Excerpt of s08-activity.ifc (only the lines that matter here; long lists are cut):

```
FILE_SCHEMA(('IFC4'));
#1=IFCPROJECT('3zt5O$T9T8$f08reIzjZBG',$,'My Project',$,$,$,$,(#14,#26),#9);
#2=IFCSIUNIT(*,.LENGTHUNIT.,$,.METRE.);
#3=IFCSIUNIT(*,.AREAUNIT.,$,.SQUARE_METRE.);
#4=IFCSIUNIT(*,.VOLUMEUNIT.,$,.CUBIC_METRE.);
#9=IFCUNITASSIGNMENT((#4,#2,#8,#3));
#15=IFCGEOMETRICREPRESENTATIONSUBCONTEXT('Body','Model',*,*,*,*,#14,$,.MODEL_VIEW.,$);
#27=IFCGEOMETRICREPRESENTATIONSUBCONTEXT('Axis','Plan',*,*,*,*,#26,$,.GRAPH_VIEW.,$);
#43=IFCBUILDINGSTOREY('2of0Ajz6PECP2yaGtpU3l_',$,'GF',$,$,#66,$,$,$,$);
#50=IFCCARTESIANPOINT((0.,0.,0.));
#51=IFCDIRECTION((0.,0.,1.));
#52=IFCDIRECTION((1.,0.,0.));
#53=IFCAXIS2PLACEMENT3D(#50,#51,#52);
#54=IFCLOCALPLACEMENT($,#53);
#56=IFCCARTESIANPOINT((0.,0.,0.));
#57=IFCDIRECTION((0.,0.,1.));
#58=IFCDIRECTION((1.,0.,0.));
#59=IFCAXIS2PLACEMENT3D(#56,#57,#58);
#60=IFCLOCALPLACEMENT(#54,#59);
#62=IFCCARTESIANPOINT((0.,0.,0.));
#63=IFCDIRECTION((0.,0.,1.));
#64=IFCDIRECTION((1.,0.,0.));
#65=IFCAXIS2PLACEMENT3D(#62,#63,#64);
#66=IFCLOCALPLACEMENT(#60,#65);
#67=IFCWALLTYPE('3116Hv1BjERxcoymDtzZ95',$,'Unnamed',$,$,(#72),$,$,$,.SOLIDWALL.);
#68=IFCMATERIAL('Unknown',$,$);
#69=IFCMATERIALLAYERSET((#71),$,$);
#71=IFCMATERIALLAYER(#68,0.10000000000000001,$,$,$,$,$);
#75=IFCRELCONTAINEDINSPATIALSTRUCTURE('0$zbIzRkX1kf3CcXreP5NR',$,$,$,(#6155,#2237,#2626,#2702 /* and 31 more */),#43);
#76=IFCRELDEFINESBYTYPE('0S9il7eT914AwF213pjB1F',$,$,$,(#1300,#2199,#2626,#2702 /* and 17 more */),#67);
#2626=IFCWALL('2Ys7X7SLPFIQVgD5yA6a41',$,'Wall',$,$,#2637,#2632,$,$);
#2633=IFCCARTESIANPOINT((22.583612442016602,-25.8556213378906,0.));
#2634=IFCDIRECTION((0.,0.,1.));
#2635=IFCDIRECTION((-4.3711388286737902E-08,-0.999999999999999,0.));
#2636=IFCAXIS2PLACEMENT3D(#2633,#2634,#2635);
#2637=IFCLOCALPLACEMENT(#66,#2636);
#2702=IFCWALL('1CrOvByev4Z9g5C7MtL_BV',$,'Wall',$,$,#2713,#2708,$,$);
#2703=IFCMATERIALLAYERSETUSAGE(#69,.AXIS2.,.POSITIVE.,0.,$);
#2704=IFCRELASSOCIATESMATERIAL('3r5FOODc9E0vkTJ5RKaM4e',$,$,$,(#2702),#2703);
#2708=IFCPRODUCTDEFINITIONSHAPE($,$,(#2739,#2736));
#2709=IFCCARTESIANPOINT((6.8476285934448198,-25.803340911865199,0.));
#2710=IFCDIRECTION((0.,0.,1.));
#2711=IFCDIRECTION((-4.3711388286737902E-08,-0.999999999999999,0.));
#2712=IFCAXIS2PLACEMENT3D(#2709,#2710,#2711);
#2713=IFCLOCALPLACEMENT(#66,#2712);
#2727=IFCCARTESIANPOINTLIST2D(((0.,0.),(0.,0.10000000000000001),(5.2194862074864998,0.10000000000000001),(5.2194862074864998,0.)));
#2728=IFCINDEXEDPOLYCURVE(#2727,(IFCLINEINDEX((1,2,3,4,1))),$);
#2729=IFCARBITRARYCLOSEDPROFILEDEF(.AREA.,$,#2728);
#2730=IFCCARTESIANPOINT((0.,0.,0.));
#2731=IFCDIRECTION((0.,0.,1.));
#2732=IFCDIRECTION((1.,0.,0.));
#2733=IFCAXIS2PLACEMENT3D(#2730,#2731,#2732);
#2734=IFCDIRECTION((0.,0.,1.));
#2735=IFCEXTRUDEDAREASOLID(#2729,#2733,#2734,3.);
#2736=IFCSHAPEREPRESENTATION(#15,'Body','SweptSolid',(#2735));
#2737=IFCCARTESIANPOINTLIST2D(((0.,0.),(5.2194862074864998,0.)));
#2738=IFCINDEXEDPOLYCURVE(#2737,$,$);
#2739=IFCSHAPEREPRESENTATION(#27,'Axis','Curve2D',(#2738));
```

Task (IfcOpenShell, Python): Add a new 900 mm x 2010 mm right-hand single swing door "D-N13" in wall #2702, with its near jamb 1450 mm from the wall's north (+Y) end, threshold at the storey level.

```python
import numpy as np
import ifcopenshell
import ifcopenshell.api.feature
import ifcopenshell.api.geometry
import ifcopenshell.api.root
import ifcopenshell.api.spatial
import ifcopenshell.geom
import ifcopenshell.util.element
import ifcopenshell.util.placement
import ifcopenshell.util.representation
import ifcopenshell.util.shape
import ifcopenshell.util.unit

model = ifcopenshell.open("s08-activity.ifc")
unit_scale = ifcopenshell.util.unit.calculate_unit_scale(model)
settings = ifcopenshell.geom.settings()


def volume(element):
    """Net volume in cubic metres, openings subtracted."""
    shape = ifcopenshell.geom.create_shape(settings, element)
    return ifcopenshell.util.shape.get_volume(shape.geometry)


wall = model.by_guid("1CrOvByev4Z9g5C7MtL_BV")
storey = ifcopenshell.util.element.get_container(wall, ifc_class="IfcBuildingStorey")
context = ifcopenshell.util.representation.get_context(model, "Model", "Body", "MODEL_VIEW")
before = volume(wall)

width, height, from_end, sill = 0.9, 2.01, 1.45, 0.0  # metres

# The wall runs along its own X axis, and the end named is its -X end.
wall_shape = ifcopenshell.geom.create_shape(settings, wall)
x, y, z = ifcopenshell.util.shape.get_vertices(wall_shape.geometry).T
start = x.min() + from_end
face, thickness = float(y.min()), float(y.max() - y.min())
wall_matrix = ifcopenshell.util.placement.get_local_placement(wall.ObjectPlacement)
level = ifcopenshell.util.placement.get_local_placement(storey.ObjectPlacement)[2, 3]


def in_wall(x, y):
    """Placement at x, y metres in the wall's axes, at sill height."""
    matrix = wall_matrix.copy()
    matrix[:, 3] = wall_matrix @ np.array([x / unit_scale, y / unit_scale, 0.0, 1.0])
    matrix[2, 3] = level + sill / unit_scale
    return matrix


# Opening: a box that overshoots both wall faces by 50 mm.
opening = ifcopenshell.api.root.create_entity(model, ifc_class="IfcOpeningElement", predefined_type="OPENING")
box = ifcopenshell.api.geometry.add_wall_representation(
    model, context=context, length=width, height=height, thickness=thickness + 0.1
)
ifcopenshell.api.geometry.assign_representation(model, product=opening, representation=box)
ifcopenshell.api.geometry.edit_object_placement(model, product=opening, matrix=in_wall(start, face - 0.05), is_si=False)
ifcopenshell.api.feature.add_feature(model, feature=opening, element=wall)

door = ifcopenshell.api.root.create_entity(model, ifc_class="IfcDoor", name="D-N13", predefined_type="DOOR")
door.OverallWidth, door.OverallHeight = width / unit_scale, height / unit_scale
door.OperationType = "SINGLE_SWING_RIGHT"
body = ifcopenshell.api.geometry.add_door_representation(
    model,
    context=context,
    overall_width=door.OverallWidth,
    overall_height=door.OverallHeight,
    operation_type="SINGLE_SWING_RIGHT",
    lining_properties={"LiningDepth": thickness / unit_scale, "ThresholdDepth": thickness / unit_scale},
)
ifcopenshell.api.geometry.assign_representation(model, product=door, representation=body)
ifcopenshell.api.spatial.assign_container(model, products=[door], relating_structure=storey)
ifcopenshell.api.feature.add_filling(model, opening=opening, element=door)

# The lining spans the wall, so the door starts at the wall face.
ifcopenshell.api.geometry.edit_object_placement(model, product=door, matrix=in_wall(start, face), is_si=False)

after = volume(wall)

print(f"wall volume {before:.3f} -> {after:.3f} m3")

model.write("s08-activity_updated.ifc")
```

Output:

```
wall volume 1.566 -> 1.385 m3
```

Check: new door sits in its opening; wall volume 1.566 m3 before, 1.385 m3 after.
